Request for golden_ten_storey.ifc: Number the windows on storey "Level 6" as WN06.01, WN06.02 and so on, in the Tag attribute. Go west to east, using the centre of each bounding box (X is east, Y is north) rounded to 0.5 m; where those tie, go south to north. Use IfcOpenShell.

First a look at what the model holds.

```python
import ifcopenshell
import ifcopenshell.util.element
import ifcopenshell.util.placement

model = ifcopenshell.open("golden_ten_storey.ifc")
print(model.schema)
storey = next(s for s in model.by_type("IfcBuildingStorey") if s.Name == "Level 6")
windows = [e for e in ifcopenshell.util.element.get_decomposition(storey) if e.is_a("IfcWindow")]
for e in sorted(windows, key=lambda e: e.id()):
    origin = ifcopenshell.util.placement.get_local_placement(e.ObjectPlacement)[:3, 3]
    print(e.id(), e.Tag, e.Name, origin.round(2) + 0.0, sep=" | ")
```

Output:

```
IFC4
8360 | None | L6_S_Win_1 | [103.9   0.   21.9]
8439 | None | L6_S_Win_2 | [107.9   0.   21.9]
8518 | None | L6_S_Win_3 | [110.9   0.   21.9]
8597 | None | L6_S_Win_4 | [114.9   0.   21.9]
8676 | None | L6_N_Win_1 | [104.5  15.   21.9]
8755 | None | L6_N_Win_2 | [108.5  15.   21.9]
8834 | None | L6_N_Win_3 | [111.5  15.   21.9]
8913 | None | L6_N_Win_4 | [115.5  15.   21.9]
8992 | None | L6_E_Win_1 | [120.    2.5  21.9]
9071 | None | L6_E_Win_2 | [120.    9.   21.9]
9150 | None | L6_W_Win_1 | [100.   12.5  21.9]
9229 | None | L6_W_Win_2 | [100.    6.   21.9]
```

```python
import ifcopenshell
import ifcopenshell.geom
import ifcopenshell.util.element
import ifcopenshell.util.shape

model = ifcopenshell.open("golden_ten_storey.ifc")
settings = ifcopenshell.geom.settings()
settings.set("use-world-coords", True)


def centre(element):
    shape = ifcopenshell.geom.create_shape(settings, element)
    return ifcopenshell.util.shape.get_bbox_centroid(shape.geometry)


storey = next(s for s in model.by_type("IfcBuildingStorey") if s.Name == "Level 6")
windows = [e for e in ifcopenshell.util.element.get_decomposition(storey) if e.is_a("IfcWindow")]

# Insertion points can sit at a corner or the storey origin, so sort by the geometry (in metres).
centres = {e: centre(e) for e in windows}
windows.sort(key=lambda e: (round(centres[e][0] / 0.5), centres[e][1]))

for i, e in enumerate(windows, start=1):
    number = f"WN06.{i:02d}"
    e.Tag = number
    print(e.id(), number)

model.write("golden_ten_storey_edited.ifc")
```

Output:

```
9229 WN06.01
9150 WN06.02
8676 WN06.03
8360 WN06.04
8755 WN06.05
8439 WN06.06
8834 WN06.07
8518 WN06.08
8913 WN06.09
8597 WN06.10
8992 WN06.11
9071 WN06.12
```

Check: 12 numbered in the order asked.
